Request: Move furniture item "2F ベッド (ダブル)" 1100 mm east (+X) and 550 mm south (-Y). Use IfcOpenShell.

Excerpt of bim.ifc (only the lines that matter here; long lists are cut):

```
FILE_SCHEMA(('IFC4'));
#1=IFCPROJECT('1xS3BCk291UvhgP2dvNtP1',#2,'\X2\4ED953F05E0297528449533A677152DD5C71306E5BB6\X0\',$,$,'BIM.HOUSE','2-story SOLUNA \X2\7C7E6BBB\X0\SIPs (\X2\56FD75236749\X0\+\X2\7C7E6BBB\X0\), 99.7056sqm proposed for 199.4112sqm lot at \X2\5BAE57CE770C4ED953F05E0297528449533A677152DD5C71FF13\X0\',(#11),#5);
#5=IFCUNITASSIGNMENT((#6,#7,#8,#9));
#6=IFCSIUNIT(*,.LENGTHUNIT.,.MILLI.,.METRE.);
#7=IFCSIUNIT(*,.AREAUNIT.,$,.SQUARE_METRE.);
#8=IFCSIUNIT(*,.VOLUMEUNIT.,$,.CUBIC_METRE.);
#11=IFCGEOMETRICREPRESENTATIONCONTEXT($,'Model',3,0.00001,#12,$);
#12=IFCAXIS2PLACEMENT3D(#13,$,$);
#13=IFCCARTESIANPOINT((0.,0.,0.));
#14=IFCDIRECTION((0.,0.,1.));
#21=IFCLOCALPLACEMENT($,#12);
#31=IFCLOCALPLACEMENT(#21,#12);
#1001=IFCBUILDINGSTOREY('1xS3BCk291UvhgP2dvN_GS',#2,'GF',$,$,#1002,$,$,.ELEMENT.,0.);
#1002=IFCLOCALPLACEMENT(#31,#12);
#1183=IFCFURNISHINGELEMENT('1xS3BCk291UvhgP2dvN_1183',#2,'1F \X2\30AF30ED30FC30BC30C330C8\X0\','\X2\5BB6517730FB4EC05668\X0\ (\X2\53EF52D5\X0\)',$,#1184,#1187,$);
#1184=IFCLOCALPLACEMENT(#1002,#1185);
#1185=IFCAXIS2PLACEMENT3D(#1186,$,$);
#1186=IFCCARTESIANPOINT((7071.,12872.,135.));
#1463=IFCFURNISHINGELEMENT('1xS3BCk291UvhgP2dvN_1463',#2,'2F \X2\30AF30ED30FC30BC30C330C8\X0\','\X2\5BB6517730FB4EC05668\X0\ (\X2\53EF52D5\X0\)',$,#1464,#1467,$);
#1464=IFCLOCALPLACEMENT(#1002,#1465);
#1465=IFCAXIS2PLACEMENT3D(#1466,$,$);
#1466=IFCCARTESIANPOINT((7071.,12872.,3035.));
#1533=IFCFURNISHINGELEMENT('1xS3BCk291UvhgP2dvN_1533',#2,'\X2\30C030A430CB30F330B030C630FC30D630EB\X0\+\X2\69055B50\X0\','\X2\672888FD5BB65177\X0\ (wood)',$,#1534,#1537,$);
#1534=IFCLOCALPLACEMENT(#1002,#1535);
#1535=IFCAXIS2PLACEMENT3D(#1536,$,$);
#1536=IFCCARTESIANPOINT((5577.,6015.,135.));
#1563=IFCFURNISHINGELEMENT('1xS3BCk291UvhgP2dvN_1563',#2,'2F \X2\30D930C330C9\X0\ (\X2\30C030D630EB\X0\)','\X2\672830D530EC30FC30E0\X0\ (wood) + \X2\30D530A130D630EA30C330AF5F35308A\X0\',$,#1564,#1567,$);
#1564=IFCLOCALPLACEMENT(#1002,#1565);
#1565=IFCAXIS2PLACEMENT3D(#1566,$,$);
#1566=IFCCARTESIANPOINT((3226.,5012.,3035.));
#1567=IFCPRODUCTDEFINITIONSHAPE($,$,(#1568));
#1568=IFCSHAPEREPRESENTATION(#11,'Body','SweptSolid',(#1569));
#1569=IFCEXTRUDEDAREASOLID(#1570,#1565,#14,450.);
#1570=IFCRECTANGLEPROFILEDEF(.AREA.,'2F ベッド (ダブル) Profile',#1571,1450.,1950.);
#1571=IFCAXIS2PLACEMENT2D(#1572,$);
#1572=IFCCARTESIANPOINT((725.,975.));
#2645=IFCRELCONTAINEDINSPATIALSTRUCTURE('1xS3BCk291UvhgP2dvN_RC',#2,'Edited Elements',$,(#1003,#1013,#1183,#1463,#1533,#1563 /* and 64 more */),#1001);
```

```python
import ifcopenshell
import ifcopenshell.api.geometry
import ifcopenshell.util.placement

model = ifcopenshell.open("bim.ifc")

item = model.by_id(1563)
matrix = ifcopenshell.util.placement.get_local_placement(item.ObjectPlacement)
matrix[0, 3] += 1100.0
matrix[1, 3] -= 550.0
ifcopenshell.api.geometry.edit_object_placement(model, product=item, matrix=matrix, is_si=False)

print(ifcopenshell.util.placement.get_local_placement(item.ObjectPlacement).round(3) + 0.0)

model.write("bim_edited.ifc")
```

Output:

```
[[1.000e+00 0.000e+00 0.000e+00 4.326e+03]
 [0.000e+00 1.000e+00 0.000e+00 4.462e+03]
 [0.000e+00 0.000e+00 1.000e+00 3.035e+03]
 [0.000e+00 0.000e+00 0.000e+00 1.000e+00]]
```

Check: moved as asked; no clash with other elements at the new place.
